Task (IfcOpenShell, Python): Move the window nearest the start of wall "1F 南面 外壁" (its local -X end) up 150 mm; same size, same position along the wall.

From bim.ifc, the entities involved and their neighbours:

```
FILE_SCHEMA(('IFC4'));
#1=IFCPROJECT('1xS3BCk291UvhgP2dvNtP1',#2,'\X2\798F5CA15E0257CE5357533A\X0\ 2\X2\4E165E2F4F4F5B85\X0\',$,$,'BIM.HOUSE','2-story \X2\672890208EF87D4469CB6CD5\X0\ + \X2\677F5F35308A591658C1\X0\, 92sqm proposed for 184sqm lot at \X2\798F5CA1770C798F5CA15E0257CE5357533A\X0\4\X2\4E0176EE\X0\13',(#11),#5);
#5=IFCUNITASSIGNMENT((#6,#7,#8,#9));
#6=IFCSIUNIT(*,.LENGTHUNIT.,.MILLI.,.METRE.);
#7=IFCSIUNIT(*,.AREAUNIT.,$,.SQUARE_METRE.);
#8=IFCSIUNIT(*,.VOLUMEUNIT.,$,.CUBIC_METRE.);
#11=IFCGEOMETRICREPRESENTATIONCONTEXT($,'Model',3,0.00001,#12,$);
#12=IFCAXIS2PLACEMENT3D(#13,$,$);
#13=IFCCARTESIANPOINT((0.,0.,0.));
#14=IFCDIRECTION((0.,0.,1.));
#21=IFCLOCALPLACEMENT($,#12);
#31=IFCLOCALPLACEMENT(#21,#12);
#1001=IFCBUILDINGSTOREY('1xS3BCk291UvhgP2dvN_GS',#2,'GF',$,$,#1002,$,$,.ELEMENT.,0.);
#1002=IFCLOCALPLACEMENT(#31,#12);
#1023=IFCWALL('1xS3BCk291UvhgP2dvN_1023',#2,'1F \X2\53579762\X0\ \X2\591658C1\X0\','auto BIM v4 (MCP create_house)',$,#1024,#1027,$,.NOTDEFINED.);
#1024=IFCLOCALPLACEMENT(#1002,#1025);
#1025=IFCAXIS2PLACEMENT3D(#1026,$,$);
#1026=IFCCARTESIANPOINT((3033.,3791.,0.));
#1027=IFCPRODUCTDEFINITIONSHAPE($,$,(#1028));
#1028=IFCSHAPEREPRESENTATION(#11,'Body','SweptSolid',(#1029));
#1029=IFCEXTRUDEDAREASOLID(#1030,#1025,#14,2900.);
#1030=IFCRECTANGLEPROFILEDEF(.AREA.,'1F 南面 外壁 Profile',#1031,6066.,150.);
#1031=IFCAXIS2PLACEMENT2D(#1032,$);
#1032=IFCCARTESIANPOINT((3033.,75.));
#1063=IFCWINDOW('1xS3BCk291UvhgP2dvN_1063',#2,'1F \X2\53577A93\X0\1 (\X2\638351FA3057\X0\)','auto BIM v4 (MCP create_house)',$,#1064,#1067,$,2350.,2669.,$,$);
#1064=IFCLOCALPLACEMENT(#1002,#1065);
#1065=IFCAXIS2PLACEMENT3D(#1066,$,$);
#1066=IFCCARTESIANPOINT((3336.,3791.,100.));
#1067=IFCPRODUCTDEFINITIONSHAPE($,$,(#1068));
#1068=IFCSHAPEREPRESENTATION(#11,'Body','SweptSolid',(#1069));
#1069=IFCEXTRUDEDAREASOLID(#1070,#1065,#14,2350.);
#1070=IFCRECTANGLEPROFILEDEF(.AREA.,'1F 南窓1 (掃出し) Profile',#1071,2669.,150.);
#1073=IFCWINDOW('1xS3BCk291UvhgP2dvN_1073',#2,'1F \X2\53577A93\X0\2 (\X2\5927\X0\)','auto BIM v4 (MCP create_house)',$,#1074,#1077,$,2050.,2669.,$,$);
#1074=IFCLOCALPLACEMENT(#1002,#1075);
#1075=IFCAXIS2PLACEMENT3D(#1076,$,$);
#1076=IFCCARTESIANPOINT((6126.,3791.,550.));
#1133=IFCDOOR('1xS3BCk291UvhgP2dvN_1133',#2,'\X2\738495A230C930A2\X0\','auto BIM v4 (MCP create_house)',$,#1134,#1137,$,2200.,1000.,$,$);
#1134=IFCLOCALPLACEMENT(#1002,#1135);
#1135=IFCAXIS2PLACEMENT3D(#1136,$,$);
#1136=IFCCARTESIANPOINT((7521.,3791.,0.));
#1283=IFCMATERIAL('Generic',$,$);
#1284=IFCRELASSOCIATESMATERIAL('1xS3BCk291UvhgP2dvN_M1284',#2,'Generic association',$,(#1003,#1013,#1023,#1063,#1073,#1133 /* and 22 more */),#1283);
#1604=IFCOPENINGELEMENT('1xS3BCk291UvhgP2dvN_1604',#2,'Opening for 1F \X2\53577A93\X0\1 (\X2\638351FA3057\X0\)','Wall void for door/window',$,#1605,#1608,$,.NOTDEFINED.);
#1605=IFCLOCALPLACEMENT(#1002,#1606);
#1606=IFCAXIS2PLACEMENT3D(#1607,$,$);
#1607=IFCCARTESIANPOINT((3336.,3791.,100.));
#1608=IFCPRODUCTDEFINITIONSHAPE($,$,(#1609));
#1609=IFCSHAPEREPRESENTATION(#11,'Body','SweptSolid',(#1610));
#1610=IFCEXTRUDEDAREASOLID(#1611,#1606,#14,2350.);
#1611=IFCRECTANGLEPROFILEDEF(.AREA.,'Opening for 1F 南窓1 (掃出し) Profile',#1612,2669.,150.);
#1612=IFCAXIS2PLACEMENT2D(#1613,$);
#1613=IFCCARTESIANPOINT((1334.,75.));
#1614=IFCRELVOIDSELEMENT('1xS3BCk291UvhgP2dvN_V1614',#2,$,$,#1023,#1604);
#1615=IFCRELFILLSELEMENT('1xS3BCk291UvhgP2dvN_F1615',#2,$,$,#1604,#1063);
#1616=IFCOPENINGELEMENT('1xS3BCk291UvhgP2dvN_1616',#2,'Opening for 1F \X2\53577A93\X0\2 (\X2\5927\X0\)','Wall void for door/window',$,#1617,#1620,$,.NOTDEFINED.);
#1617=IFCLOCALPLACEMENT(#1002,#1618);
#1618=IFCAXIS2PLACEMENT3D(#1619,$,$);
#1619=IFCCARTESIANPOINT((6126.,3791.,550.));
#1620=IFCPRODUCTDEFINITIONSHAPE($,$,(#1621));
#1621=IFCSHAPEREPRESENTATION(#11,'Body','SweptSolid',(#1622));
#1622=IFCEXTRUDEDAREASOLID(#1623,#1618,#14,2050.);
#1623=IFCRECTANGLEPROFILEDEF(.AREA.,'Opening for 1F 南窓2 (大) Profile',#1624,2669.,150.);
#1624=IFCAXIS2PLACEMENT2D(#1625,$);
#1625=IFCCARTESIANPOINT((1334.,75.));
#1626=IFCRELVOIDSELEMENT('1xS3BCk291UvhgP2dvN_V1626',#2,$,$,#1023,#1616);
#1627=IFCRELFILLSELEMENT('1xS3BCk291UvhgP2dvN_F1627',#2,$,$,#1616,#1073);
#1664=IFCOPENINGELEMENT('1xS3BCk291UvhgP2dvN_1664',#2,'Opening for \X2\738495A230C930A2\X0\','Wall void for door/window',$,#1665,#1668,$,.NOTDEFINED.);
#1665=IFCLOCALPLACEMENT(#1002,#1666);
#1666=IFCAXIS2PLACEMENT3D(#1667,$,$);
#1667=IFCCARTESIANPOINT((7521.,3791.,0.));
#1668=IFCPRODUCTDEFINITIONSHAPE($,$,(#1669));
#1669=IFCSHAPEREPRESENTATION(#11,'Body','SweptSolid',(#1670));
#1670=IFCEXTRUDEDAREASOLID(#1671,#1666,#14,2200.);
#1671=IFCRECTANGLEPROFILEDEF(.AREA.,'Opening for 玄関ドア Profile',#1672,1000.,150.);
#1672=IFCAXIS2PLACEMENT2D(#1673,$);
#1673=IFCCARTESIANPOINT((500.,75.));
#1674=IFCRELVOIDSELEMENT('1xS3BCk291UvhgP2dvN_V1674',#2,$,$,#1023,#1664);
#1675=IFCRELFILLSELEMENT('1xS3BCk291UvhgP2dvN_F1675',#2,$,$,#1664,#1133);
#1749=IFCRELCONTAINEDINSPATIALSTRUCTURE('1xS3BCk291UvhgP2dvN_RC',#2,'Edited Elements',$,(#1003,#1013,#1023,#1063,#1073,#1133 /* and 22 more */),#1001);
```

```python
import numpy as np
import ifcopenshell
import ifcopenshell.api.geometry
import ifcopenshell.util.placement
import ifcopenshell.util.unit

model = ifcopenshell.open("bim.ifc")
unit_scale = ifcopenshell.util.unit.calculate_unit_scale(model)

window = model.by_id(1063)
opening = window.FillsVoids[0].RelatingOpeningElement
dz = 150.0

shift = np.array([0.0, 0.0, dz])
# The window is not placed relative to its opening, so move both.
for product in (opening, window):
    matrix = ifcopenshell.util.placement.get_local_placement(product.ObjectPlacement)
    matrix[:3, 3] += shift
    ifcopenshell.api.geometry.edit_object_placement(model, product=product, matrix=matrix, is_si=False)

print(f"moved by {dz * unit_scale:+.3f} m")

model.write("bim_v2.ifc")
```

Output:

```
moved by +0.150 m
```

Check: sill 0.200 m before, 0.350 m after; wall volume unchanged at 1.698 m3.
